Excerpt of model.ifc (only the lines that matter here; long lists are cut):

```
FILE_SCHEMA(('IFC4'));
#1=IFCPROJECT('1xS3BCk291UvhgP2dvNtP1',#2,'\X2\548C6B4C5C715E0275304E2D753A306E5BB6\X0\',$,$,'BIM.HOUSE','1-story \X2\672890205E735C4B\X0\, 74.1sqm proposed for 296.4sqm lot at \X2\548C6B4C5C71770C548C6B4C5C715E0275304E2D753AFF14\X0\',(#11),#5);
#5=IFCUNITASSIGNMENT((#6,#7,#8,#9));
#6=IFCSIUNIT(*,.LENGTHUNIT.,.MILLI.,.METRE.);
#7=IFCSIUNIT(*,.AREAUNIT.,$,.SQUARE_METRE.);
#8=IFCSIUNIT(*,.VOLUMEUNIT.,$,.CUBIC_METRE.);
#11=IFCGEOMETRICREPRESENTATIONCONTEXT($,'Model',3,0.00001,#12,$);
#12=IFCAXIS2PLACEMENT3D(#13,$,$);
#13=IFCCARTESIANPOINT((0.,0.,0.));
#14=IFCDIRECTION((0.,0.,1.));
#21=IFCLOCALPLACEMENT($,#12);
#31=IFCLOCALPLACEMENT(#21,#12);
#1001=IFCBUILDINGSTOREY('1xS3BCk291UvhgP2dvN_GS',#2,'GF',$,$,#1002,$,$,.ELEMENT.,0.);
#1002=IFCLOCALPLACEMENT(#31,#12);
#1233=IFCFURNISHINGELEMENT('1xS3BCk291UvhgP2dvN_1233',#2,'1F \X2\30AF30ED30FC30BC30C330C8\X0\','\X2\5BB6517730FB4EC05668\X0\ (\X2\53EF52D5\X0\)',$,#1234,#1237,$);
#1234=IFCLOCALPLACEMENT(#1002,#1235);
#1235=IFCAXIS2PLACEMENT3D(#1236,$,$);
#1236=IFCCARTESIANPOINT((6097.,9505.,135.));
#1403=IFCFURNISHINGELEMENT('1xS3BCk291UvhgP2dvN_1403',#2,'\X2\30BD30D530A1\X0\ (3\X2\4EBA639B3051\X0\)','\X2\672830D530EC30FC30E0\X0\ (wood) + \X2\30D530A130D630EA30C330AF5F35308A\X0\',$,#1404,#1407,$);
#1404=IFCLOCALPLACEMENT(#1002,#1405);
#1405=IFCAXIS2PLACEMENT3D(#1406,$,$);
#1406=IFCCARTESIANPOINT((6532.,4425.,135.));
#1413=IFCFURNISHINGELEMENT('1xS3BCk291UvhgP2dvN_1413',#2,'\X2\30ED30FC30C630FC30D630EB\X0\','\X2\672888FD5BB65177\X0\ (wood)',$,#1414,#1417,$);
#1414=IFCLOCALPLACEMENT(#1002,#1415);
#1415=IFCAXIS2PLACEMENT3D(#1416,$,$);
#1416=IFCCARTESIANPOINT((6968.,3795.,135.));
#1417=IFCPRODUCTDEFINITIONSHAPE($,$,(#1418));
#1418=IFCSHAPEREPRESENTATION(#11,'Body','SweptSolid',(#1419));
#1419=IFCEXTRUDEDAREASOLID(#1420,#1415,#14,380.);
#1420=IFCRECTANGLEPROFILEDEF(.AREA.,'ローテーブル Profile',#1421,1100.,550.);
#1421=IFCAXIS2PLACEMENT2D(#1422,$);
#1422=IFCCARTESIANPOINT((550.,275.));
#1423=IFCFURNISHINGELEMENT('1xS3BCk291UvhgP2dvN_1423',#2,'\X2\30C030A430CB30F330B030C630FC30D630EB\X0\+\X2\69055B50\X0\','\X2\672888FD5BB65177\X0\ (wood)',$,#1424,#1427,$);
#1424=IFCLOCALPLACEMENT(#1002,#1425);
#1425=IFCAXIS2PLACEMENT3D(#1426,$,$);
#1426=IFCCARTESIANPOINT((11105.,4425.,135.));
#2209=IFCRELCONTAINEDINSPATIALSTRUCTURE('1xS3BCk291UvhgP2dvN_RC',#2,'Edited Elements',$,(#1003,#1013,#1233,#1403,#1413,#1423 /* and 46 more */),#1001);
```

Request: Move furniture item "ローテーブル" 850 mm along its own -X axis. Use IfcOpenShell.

```python
import ifcopenshell
import ifcopenshell.api.geometry
import ifcopenshell.util.placement

model = ifcopenshell.open("model.ifc")

item = model.by_guid("1xS3BCk291UvhgP2dvN_1413")
matrix = ifcopenshell.util.placement.get_local_placement(item.ObjectPlacement)
matrix[:3, 3] -= matrix[:3, 0] * 850.0
ifcopenshell.api.geometry.edit_object_placement(model, product=item, matrix=matrix, is_si=False)

print(ifcopenshell.util.placement.get_local_placement(item.ObjectPlacement).round(3) + 0.0)

model.write("model_updated.ifc")
```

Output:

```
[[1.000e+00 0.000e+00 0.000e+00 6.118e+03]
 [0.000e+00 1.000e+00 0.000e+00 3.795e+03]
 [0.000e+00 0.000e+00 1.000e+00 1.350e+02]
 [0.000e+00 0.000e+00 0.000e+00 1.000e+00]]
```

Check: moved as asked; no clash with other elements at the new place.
